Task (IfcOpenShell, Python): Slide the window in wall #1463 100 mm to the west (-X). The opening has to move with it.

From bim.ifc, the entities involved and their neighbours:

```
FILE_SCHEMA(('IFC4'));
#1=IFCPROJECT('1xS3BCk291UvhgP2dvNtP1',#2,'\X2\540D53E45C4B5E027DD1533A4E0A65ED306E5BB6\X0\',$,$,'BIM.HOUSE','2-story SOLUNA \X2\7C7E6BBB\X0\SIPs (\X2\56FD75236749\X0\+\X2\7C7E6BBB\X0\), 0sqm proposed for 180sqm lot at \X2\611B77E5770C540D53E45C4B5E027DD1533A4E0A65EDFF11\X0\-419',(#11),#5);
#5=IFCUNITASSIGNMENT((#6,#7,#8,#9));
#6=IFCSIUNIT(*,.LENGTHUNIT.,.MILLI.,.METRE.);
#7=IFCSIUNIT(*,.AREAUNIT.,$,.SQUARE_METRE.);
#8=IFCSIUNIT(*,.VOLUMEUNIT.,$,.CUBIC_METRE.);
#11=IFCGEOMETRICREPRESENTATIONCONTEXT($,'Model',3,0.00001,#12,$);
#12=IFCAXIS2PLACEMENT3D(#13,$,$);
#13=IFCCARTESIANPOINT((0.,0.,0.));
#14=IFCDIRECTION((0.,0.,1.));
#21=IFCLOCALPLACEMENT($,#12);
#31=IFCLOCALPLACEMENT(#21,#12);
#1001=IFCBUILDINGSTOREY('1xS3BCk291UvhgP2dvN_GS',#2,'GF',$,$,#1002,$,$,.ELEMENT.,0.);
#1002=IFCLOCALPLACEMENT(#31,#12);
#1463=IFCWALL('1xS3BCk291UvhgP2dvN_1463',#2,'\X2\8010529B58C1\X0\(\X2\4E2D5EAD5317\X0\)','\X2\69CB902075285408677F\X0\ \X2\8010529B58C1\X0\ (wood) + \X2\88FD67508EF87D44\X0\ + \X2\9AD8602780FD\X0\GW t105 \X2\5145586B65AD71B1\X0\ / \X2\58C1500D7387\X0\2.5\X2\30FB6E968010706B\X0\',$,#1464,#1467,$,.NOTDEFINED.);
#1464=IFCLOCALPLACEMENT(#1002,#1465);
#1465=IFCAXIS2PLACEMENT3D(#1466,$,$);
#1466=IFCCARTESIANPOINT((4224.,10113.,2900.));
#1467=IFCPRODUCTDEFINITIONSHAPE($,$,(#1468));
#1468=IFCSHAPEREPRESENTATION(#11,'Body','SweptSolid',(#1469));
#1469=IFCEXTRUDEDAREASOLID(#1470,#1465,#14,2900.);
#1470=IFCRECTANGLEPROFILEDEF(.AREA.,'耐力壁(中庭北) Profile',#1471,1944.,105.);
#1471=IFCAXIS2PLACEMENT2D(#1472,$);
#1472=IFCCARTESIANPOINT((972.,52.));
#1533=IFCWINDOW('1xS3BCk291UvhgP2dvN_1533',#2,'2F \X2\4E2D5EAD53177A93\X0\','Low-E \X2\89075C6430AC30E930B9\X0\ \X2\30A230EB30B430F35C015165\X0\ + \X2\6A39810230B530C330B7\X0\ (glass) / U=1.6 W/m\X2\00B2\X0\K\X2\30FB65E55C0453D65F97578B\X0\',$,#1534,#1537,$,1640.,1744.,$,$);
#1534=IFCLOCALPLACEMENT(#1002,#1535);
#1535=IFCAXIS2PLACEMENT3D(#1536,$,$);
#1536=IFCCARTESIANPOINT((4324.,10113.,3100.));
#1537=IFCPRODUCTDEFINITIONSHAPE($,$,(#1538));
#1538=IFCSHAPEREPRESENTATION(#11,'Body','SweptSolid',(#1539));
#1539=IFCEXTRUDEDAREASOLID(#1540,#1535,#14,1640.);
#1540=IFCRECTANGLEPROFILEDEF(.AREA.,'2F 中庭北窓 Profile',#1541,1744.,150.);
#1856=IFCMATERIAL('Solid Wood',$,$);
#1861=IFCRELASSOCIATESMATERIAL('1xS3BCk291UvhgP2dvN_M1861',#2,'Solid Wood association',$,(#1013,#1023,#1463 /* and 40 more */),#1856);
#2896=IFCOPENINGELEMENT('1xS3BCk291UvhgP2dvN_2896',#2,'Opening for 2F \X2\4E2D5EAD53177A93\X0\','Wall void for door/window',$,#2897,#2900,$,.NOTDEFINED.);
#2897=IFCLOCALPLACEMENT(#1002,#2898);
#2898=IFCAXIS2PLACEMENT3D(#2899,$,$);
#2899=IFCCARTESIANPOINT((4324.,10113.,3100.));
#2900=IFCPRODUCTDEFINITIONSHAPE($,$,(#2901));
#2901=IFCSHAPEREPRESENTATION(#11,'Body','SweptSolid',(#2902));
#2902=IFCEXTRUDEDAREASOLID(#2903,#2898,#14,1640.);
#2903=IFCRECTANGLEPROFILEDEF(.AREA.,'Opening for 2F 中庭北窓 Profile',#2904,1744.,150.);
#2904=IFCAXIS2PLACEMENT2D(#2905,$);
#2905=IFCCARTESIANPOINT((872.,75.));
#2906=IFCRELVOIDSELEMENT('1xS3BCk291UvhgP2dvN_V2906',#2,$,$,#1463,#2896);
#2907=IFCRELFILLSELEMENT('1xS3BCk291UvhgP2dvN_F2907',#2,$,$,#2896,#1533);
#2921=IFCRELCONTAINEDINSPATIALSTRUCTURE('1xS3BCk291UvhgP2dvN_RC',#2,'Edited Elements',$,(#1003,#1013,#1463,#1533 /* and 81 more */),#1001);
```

```python
import ifcopenshell
import ifcopenshell.api.geometry
import ifcopenshell.util.placement
import ifcopenshell.util.unit

model = ifcopenshell.open("bim.ifc")
unit_scale = ifcopenshell.util.unit.calculate_unit_scale(model)

window = model.by_guid("1xS3BCk291UvhgP2dvN_1533")
opening = window.FillsVoids[0].RelatingOpeningElement
wall = opening.VoidsElements[0].RelatingBuildingElement

wall_matrix = ifcopenshell.util.placement.get_local_placement(wall.ObjectPlacement)
shift = wall_matrix[:3, 0] * -0.1 / unit_scale
before = ifcopenshell.util.placement.get_local_placement(window.ObjectPlacement)[:3, 3].copy()

# The window is not placed relative to its opening, so move both.
for product in (opening, window):
    matrix = ifcopenshell.util.placement.get_local_placement(product.ObjectPlacement)
    matrix[:3, 3] += shift
    ifcopenshell.api.geometry.edit_object_placement(model, product=product, matrix=matrix, is_si=False)

after = ifcopenshell.util.placement.get_local_placement(window.ObjectPlacement)[:3, 3]
print("window moved by", (after - before).round(3) + 0.0)

model.write("bim_edited.ifc")
```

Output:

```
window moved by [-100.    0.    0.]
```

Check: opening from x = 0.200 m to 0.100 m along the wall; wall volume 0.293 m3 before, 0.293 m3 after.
